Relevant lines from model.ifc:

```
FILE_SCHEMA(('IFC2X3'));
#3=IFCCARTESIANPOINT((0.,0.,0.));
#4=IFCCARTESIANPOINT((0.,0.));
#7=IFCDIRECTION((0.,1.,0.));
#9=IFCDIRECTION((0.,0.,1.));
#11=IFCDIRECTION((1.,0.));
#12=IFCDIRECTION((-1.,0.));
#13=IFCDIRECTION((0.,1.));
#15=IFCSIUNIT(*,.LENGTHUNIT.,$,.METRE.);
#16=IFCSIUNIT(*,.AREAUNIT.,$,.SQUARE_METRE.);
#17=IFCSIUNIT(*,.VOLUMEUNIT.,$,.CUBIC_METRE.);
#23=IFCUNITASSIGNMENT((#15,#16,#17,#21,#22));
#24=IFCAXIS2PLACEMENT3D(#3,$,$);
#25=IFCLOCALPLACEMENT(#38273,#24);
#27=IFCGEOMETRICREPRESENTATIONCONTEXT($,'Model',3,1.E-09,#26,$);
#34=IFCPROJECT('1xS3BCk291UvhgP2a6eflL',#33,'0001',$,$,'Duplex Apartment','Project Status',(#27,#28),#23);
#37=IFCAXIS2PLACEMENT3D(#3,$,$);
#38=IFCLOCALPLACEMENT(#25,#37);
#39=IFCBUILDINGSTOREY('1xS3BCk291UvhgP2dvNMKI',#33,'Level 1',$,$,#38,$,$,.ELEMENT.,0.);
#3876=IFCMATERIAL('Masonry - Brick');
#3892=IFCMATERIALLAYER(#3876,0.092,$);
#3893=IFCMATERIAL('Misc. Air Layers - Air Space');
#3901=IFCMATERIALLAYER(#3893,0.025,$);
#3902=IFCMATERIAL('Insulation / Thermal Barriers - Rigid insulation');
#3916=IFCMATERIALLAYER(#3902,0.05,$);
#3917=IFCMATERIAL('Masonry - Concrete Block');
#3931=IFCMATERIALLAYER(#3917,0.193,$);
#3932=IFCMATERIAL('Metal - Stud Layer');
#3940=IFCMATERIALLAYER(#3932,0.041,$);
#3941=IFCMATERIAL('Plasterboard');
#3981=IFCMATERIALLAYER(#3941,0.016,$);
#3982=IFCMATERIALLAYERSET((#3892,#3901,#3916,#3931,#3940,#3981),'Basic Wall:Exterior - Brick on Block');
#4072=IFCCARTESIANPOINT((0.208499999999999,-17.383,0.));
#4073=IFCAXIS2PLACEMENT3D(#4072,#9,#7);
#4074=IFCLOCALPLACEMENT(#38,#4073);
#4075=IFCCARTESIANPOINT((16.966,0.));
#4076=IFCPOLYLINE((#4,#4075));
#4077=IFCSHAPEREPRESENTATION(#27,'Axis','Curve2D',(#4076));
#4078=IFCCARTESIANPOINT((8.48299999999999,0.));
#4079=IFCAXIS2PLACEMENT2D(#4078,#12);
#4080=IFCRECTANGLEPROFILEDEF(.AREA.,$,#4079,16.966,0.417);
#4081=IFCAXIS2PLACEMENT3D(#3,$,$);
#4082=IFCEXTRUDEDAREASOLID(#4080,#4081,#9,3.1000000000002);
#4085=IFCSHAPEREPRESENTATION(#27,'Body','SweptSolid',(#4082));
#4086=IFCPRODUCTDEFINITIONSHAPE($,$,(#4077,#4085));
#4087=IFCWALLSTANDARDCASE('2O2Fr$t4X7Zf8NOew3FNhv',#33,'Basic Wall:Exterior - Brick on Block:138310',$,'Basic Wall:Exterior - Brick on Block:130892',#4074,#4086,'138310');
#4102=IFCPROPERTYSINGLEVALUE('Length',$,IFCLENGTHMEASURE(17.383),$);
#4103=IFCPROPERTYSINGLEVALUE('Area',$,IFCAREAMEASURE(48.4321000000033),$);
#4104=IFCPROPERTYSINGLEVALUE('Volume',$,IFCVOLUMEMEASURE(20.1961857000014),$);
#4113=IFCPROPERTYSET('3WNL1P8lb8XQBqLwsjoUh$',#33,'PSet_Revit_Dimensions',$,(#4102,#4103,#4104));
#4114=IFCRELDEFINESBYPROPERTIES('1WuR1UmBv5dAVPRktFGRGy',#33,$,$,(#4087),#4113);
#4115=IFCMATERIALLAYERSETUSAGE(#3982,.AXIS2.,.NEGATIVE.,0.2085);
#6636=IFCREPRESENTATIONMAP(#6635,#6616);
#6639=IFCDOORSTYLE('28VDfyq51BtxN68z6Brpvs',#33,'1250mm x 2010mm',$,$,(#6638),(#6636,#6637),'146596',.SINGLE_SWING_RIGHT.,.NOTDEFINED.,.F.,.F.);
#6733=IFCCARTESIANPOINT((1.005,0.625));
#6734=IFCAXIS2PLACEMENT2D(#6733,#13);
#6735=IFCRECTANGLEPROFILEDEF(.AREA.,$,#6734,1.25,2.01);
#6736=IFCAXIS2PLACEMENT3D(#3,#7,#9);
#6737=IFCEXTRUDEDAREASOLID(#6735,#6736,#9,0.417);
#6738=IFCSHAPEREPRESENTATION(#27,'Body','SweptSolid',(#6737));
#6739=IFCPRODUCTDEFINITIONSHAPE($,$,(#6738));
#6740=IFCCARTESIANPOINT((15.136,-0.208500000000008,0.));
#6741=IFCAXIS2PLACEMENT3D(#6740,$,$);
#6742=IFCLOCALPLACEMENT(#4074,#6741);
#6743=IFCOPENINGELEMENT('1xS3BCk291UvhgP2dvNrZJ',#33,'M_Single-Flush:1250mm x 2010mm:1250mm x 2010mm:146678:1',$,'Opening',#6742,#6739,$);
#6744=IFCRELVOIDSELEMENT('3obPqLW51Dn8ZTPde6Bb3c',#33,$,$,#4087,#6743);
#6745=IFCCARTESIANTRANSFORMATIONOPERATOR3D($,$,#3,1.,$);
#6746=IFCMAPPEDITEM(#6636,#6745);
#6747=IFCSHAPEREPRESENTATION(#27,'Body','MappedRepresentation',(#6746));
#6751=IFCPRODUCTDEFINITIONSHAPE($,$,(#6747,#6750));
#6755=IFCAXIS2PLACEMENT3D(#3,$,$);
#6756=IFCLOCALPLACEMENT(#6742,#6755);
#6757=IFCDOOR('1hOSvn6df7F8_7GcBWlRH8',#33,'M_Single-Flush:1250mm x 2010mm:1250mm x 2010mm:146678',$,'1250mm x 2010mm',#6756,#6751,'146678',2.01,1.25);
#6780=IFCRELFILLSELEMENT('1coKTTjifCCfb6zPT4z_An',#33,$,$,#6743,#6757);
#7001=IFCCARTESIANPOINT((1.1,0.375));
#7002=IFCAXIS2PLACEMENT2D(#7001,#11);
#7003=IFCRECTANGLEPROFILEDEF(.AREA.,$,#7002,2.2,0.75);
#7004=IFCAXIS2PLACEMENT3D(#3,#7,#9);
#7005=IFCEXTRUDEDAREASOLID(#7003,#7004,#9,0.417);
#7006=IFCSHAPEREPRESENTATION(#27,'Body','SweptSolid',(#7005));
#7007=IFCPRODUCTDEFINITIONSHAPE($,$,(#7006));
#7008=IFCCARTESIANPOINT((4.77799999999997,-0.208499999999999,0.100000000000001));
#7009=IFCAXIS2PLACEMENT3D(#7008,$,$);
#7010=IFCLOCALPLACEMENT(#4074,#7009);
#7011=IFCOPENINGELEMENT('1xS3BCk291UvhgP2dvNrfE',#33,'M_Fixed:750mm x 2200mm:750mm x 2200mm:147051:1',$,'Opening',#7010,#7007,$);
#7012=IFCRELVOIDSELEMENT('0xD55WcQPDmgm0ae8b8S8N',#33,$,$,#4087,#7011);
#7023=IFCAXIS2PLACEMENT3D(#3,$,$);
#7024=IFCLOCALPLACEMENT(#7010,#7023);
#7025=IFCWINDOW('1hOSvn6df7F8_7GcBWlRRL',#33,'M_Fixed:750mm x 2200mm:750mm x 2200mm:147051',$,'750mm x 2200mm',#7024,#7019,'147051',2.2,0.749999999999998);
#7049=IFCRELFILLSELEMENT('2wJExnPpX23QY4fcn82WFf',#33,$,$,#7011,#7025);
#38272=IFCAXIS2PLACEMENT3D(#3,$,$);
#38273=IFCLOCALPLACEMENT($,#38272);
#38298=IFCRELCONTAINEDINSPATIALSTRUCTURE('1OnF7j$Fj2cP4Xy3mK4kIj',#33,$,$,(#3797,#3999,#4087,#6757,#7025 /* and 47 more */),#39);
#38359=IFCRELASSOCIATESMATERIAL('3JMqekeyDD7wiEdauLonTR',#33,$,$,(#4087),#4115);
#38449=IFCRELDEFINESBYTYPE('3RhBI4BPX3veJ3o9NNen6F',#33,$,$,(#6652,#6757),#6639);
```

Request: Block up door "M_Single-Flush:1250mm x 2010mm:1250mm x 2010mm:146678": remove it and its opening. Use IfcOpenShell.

```python
import ifcopenshell
import ifcopenshell.api.feature
import ifcopenshell.api.pset
import ifcopenshell.api.root
import ifcopenshell.geom
import ifcopenshell.util.element
import ifcopenshell.util.shape
import ifcopenshell.util.unit

model = ifcopenshell.open("model.ifc")
area_scale = ifcopenshell.util.unit.calculate_unit_scale(model, "AREAUNIT")
volume_scale = ifcopenshell.util.unit.calculate_unit_scale(model, "VOLUMEUNIT")
settings = ifcopenshell.geom.settings()


def volume(element):
    """Net volume in cubic metres, openings subtracted."""
    shape = ifcopenshell.geom.create_shape(settings, element)
    return ifcopenshell.util.shape.get_volume(shape.geometry)


door = model.by_guid("1hOSvn6df7F8_7GcBWlRH8")
opening = door.FillsVoids[0].RelatingOpeningElement
wall = opening.VoidsElements[0].RelatingBuildingElement
before = volume(wall)

ifcopenshell.api.root.remove_product(model, product=door)
ifcopenshell.api.feature.remove_feature(model, feature=opening)

after = volume(wall)
thickness = 0.417  # wall thickness in metres

# Update the wall's stored quantities.
pset = model.by_id(ifcopenshell.util.element.get_pset(wall, "PSet_Revit_Dimensions", should_inherit=False)["id"])
ifcopenshell.api.pset.edit_pset(model, pset=pset, properties={
    "Area": model.create_entity("IfcAreaMeasure", after / thickness / area_scale),
    "Volume": model.create_entity("IfcVolumeMeasure", after / volume_scale),
})

print(f"wall volume {before:.3f} -> {after:.3f} m3")

model.write("model-out.ifc")
```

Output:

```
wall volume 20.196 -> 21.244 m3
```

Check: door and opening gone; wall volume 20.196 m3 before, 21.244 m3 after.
